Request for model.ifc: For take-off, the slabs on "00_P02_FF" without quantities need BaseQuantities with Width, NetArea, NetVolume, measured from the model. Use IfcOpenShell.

First a look at what the model holds.

```python
import ifcopenshell
import ifcopenshell.util.element
import ifcopenshell.util.unit

model = ifcopenshell.open("model.ifc")
print(model.schema)
for unit_type in ("LENGTHUNIT", "AREAUNIT", "VOLUMEUNIT"):
    print(unit_type, ifcopenshell.util.unit.calculate_unit_scale(model, unit_type))
storey = next(s for s in model.by_type("IfcBuildingStorey") if s.Name == "00_P02_FF")
slabs = [e for e in ifcopenshell.util.element.get_decomposition(storey) if e.is_a("IfcSlab")]
for e in sorted(slabs, key=lambda e: e.id()):
    print(e.id(), e.is_a(), e.Name, list(ifcopenshell.util.element.get_psets(e, qtos_only=True)), sep=" | ")
```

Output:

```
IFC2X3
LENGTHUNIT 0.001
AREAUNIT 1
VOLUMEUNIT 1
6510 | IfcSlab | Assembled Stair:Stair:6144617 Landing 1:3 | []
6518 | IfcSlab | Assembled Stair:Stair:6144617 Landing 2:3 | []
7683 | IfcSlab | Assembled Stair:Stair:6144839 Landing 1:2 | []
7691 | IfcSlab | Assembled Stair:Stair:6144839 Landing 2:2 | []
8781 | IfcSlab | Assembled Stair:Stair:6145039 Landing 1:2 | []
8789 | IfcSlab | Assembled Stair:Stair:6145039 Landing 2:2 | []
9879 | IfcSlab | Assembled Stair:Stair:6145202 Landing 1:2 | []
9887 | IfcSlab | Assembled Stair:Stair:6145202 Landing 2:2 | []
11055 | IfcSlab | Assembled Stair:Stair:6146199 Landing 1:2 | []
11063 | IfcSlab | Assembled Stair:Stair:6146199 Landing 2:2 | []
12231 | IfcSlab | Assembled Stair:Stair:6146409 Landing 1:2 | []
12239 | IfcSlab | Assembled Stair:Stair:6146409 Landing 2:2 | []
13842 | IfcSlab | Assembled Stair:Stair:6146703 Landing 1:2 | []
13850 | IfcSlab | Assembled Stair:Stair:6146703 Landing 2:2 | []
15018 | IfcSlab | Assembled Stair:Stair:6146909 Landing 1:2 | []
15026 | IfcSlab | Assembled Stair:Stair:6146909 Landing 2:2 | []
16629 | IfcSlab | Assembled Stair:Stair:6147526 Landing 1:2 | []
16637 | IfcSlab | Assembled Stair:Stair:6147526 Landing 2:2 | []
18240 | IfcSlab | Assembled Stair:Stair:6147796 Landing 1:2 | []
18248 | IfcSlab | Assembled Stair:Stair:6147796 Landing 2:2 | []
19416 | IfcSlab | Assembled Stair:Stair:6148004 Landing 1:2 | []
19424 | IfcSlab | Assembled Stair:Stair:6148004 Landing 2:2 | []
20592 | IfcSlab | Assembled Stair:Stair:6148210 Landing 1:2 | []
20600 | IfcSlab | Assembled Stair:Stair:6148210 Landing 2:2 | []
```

```python
import ifcopenshell
import ifcopenshell.api.pset
import ifcopenshell.geom
import ifcopenshell.util.element
import ifcopenshell.util.shape
import ifcopenshell.util.unit

model = ifcopenshell.open("model.ifc")
unit_scale = ifcopenshell.util.unit.calculate_unit_scale(model)
area_scale = ifcopenshell.util.unit.calculate_unit_scale(model, "AREAUNIT")
volume_scale = ifcopenshell.util.unit.calculate_unit_scale(model, "VOLUMEUNIT")
settings = ifcopenshell.geom.settings()

storey = next(s for s in model.by_type("IfcBuildingStorey") if s.Name == "00_P02_FF")
slabs = [e for e in ifcopenshell.util.element.get_decomposition(storey) if e.is_a("IfcSlab")]

for e in sorted(slabs, key=lambda e: e.id()):
    if ifcopenshell.util.element.get_psets(e, qtos_only=True, should_inherit=False):
        continue
    # Geometry comes back in metres, in the element's own axes.
    shape = ifcopenshell.geom.create_shape(settings, e)
    values = {
        "Width": ifcopenshell.util.shape.get_z(shape.geometry) / unit_scale,
        "NetArea": ifcopenshell.util.shape.get_footprint_area(shape.geometry) / area_scale,
        "NetVolume": ifcopenshell.util.shape.get_volume(shape.geometry) / volume_scale,
    }
    qto = ifcopenshell.api.pset.add_qto(model, product=e, name="BaseQuantities")
    ifcopenshell.api.pset.edit_qto(model, qto=qto, properties=values)
    print(e.id(), {k: round(v, 3) for k, v in values.items()})

model.write("model-out.ifc")
```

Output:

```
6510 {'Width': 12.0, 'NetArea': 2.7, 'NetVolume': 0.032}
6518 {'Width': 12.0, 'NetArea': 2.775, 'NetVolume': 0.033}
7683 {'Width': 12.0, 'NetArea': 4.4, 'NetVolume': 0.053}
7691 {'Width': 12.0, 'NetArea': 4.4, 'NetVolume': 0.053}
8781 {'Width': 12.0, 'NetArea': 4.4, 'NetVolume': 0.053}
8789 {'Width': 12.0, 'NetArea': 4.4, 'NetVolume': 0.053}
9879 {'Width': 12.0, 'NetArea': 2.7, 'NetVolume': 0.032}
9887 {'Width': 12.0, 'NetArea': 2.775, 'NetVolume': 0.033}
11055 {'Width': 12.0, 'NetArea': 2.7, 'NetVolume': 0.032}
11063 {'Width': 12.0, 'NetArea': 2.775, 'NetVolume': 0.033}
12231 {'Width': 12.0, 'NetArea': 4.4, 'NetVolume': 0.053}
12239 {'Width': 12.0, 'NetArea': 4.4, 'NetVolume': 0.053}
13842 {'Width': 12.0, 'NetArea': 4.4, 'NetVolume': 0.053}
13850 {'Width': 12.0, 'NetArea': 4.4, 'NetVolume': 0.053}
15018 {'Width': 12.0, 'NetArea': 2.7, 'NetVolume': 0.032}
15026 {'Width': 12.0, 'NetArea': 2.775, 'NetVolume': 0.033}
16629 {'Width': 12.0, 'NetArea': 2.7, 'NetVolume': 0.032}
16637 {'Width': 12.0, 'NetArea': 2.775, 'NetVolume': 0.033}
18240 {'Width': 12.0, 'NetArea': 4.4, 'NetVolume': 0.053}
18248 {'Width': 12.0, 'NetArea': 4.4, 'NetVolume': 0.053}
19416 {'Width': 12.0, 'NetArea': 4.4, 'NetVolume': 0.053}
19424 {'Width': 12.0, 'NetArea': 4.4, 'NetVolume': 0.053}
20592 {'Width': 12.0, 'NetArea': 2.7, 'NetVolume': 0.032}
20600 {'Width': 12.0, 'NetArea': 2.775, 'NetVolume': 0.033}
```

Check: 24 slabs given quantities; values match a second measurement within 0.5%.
